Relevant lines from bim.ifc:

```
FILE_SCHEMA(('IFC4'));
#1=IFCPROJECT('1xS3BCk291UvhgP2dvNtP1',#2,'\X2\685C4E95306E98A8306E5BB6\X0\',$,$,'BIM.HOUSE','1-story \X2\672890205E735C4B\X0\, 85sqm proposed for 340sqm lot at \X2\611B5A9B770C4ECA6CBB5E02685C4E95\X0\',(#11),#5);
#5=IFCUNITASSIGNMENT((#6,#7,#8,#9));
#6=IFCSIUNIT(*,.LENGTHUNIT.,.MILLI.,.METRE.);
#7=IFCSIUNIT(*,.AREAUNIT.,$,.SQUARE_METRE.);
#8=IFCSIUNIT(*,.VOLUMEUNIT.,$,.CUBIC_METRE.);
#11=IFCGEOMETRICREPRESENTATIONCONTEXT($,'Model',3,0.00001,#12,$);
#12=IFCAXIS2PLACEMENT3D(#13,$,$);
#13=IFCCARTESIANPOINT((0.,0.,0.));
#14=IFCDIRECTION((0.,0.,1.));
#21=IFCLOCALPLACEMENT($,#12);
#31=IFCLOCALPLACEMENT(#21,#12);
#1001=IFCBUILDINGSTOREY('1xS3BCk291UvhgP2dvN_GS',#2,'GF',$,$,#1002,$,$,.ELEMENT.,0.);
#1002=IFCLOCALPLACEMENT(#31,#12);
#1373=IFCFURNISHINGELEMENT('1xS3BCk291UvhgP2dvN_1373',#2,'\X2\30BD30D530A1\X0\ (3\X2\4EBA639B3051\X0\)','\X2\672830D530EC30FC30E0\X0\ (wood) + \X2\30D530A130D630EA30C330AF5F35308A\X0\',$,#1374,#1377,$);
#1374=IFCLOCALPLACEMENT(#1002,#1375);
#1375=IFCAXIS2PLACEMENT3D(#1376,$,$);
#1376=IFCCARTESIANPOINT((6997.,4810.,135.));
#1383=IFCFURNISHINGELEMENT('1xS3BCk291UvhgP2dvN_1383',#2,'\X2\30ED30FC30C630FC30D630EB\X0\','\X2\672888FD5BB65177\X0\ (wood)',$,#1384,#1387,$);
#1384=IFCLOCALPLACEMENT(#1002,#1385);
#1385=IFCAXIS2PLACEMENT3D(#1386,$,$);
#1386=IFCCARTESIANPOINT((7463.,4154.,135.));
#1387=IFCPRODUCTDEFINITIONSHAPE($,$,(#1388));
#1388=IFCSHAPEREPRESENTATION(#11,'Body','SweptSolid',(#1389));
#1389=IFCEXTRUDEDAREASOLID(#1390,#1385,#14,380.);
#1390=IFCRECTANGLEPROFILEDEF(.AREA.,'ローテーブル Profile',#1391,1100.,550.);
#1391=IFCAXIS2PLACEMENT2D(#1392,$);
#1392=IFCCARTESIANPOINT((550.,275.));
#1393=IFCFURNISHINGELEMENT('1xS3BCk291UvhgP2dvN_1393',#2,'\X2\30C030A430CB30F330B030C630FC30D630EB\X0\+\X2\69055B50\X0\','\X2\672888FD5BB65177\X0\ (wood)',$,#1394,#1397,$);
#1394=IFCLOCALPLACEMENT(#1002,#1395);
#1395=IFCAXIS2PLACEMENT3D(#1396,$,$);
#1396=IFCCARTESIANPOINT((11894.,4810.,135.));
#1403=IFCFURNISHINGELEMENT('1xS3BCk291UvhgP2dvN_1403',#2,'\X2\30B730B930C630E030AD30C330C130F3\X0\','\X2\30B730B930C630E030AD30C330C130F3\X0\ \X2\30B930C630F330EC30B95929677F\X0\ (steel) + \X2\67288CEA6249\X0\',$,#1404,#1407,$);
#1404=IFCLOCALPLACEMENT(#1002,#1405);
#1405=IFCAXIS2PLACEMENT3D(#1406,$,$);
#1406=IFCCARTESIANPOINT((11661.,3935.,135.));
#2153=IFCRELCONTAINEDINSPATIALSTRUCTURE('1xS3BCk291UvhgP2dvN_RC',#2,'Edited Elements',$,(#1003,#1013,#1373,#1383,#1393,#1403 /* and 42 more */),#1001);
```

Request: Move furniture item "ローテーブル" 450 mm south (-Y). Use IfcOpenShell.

```python
import ifcopenshell
import ifcopenshell.api.geometry
import ifcopenshell.util.placement
import ifcopenshell.util.unit

model = ifcopenshell.open("bim.ifc")
unit_scale = ifcopenshell.util.unit.calculate_unit_scale(model)

item = model.by_guid("1xS3BCk291UvhgP2dvN_1383")
matrix = ifcopenshell.util.placement.get_local_placement(item.ObjectPlacement)
matrix[1, 3] -= 0.45 / unit_scale
ifcopenshell.api.geometry.edit_object_placement(model, product=item, matrix=matrix, is_si=False)

print(ifcopenshell.util.placement.get_local_placement(item.ObjectPlacement).round(3) + 0.0)

model.write("bim-out.ifc")
```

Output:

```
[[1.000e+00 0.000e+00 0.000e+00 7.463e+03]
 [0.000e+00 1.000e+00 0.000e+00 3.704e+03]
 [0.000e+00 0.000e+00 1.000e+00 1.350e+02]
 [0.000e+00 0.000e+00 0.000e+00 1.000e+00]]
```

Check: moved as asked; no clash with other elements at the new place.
